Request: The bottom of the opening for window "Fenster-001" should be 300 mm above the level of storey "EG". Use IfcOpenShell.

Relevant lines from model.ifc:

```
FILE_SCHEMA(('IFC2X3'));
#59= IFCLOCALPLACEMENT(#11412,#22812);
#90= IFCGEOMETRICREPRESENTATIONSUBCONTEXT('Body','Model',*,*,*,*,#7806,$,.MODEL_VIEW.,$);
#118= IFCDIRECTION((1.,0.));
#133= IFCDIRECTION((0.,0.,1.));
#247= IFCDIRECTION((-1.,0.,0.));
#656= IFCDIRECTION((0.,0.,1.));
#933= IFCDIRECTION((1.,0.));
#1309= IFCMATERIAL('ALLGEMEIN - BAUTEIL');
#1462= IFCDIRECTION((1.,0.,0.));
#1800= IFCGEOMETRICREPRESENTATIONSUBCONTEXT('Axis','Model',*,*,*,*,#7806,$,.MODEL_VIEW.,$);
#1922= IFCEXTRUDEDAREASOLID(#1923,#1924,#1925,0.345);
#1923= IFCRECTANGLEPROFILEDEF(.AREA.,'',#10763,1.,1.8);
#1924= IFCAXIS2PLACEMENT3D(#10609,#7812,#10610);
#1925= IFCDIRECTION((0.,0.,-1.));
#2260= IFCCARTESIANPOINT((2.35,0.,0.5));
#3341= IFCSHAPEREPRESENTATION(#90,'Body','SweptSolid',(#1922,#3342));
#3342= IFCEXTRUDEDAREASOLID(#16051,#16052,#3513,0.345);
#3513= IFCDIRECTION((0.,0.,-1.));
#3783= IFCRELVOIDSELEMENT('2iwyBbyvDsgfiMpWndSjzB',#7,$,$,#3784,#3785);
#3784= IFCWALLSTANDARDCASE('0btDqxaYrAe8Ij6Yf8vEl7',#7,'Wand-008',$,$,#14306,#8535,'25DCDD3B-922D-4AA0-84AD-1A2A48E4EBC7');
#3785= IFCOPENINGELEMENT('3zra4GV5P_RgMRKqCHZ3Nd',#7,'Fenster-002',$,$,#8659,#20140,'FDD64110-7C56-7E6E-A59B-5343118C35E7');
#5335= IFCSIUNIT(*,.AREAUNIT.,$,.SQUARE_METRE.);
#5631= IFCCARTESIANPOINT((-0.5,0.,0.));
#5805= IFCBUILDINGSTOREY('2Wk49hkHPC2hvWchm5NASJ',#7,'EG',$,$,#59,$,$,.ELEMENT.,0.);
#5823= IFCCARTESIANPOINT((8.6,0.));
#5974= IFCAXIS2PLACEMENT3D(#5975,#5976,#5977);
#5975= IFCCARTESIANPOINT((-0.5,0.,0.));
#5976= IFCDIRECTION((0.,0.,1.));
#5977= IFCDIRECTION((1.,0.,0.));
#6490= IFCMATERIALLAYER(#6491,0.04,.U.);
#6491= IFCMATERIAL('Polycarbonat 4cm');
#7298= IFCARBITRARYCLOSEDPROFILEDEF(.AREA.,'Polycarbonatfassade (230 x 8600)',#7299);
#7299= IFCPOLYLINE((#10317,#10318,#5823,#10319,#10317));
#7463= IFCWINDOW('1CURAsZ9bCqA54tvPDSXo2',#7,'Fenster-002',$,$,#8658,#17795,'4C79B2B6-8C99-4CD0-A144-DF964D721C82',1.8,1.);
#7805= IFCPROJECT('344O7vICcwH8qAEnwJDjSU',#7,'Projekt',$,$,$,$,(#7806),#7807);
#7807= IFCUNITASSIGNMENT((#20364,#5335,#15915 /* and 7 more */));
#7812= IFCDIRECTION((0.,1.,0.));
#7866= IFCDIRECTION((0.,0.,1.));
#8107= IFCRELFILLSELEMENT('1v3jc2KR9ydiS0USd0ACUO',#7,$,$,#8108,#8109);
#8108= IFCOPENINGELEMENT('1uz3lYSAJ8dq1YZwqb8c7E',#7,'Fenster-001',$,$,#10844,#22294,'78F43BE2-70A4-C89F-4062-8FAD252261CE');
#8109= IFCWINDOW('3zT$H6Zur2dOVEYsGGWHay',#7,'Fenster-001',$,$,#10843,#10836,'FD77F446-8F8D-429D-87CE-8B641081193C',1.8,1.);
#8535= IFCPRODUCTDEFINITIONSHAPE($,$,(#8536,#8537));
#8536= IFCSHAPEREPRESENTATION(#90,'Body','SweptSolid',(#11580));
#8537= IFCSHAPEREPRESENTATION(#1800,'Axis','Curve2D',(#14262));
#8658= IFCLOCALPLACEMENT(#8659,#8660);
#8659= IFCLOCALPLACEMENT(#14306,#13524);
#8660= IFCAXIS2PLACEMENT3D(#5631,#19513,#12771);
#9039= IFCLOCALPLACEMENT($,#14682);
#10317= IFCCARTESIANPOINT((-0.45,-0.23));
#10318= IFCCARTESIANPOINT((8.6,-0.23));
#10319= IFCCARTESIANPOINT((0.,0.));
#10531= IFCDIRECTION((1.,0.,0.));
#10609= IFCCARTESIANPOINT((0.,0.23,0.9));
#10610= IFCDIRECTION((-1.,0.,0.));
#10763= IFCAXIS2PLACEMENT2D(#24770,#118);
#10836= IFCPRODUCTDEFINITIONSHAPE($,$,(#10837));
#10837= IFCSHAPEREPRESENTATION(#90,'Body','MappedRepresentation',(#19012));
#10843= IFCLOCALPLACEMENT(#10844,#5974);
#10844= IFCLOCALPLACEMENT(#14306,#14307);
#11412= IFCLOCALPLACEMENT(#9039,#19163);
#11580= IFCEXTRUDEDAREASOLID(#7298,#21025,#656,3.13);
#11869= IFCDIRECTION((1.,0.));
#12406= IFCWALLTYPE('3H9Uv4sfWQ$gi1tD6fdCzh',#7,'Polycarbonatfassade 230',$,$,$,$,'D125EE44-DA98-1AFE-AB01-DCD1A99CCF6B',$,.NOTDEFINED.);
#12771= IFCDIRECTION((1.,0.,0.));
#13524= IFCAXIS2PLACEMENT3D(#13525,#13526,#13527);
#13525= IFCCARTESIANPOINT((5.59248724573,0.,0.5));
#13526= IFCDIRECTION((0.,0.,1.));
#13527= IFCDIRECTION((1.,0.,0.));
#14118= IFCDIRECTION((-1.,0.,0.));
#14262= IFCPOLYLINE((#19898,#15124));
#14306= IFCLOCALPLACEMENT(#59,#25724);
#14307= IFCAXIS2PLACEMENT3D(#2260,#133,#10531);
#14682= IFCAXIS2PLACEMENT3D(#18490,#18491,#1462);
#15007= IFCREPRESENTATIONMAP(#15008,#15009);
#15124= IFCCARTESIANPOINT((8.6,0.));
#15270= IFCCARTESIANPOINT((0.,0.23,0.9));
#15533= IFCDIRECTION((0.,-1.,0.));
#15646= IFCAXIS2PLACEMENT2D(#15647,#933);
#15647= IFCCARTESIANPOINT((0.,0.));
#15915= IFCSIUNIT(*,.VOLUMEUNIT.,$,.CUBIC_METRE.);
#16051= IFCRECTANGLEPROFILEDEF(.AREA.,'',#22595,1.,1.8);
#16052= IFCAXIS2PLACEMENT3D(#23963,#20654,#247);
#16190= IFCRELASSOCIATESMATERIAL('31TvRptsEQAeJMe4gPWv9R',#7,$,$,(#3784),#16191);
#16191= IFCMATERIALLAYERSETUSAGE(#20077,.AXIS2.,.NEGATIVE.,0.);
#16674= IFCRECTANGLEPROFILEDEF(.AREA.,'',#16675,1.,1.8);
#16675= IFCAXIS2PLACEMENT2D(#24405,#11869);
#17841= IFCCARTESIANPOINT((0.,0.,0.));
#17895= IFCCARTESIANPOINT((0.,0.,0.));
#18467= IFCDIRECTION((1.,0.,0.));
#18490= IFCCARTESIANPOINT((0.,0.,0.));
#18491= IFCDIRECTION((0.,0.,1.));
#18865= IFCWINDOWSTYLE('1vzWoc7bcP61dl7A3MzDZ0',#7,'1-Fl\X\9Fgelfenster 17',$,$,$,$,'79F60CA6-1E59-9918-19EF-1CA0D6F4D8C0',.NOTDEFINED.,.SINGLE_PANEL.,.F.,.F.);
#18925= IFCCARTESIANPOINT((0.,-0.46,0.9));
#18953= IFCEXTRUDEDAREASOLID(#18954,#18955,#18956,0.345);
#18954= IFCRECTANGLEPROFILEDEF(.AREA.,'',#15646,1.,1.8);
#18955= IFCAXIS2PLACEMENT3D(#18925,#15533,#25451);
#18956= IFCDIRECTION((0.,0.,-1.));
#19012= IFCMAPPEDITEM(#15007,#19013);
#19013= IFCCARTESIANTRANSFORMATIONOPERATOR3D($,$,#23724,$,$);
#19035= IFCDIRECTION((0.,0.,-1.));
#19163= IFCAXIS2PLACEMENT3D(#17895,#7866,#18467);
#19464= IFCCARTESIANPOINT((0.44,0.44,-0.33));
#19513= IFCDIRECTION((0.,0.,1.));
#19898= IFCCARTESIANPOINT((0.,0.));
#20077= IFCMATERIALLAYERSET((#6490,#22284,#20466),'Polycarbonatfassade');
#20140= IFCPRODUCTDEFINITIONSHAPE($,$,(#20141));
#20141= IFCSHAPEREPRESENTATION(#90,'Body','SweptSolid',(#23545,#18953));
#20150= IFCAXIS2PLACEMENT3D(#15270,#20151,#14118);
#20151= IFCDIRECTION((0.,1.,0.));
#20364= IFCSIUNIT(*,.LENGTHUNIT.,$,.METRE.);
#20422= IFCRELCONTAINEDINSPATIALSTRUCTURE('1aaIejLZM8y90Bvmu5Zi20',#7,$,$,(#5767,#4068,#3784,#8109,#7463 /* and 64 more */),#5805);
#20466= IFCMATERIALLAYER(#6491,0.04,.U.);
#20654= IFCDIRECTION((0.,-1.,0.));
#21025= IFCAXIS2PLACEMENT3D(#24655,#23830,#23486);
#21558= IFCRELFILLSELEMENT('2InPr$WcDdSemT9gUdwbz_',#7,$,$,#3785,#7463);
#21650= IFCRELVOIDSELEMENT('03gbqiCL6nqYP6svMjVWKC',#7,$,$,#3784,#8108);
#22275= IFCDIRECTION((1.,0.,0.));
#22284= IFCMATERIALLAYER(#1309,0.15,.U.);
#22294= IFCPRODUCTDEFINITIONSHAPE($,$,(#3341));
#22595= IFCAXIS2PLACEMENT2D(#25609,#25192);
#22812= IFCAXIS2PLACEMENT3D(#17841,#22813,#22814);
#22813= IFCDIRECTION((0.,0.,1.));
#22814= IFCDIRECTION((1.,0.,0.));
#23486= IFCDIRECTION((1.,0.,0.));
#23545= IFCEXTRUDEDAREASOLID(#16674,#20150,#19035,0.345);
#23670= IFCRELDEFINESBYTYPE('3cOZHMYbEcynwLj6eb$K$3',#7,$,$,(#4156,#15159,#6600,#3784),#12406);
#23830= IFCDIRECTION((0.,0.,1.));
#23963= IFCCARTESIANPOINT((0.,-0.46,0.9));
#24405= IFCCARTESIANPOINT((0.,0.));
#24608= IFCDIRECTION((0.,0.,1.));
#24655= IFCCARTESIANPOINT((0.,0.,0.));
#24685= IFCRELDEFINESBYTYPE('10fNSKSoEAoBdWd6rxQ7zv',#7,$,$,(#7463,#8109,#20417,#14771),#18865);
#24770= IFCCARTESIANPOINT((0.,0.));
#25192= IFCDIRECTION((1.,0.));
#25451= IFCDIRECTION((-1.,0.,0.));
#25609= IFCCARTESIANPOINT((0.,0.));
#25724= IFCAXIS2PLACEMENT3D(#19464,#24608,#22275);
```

```python
import numpy as np
import ifcopenshell
import ifcopenshell.api.geometry
import ifcopenshell.geom
import ifcopenshell.util.element
import ifcopenshell.util.placement
import ifcopenshell.util.shape
import ifcopenshell.util.unit

model = ifcopenshell.open("model.ifc")
unit_scale = ifcopenshell.util.unit.calculate_unit_scale(model)

window = model.by_id(8109)
opening = window.FillsVoids[0].RelatingOpeningElement
storey = ifcopenshell.util.element.get_container(window, ifc_class="IfcBuildingStorey")
level = ifcopenshell.util.placement.get_local_placement(storey.ObjectPlacement)[2, 3]

# The opening's origin need not be at the sill, so measure its lowest point.
shape = ifcopenshell.geom.create_shape(ifcopenshell.geom.settings(), opening)
bottom = ifcopenshell.util.shape.get_shape_bottom_elevation(shape, shape.geometry) / unit_scale
dz = level + 0.3 / unit_scale - bottom

shift = np.array([0.0, 0.0, dz])
# The window is placed relative to its opening, so it follows when the opening moves.
matrix = ifcopenshell.util.placement.get_local_placement(opening.ObjectPlacement)
matrix[:3, 3] += shift
ifcopenshell.api.geometry.edit_object_placement(
    model, product=opening, matrix=matrix, is_si=False, should_transform_children=True
)

print(f"moved by {dz * unit_scale:+.3f} m")

model.write("model_rev.ifc")
```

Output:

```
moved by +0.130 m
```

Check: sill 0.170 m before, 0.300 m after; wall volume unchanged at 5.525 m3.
